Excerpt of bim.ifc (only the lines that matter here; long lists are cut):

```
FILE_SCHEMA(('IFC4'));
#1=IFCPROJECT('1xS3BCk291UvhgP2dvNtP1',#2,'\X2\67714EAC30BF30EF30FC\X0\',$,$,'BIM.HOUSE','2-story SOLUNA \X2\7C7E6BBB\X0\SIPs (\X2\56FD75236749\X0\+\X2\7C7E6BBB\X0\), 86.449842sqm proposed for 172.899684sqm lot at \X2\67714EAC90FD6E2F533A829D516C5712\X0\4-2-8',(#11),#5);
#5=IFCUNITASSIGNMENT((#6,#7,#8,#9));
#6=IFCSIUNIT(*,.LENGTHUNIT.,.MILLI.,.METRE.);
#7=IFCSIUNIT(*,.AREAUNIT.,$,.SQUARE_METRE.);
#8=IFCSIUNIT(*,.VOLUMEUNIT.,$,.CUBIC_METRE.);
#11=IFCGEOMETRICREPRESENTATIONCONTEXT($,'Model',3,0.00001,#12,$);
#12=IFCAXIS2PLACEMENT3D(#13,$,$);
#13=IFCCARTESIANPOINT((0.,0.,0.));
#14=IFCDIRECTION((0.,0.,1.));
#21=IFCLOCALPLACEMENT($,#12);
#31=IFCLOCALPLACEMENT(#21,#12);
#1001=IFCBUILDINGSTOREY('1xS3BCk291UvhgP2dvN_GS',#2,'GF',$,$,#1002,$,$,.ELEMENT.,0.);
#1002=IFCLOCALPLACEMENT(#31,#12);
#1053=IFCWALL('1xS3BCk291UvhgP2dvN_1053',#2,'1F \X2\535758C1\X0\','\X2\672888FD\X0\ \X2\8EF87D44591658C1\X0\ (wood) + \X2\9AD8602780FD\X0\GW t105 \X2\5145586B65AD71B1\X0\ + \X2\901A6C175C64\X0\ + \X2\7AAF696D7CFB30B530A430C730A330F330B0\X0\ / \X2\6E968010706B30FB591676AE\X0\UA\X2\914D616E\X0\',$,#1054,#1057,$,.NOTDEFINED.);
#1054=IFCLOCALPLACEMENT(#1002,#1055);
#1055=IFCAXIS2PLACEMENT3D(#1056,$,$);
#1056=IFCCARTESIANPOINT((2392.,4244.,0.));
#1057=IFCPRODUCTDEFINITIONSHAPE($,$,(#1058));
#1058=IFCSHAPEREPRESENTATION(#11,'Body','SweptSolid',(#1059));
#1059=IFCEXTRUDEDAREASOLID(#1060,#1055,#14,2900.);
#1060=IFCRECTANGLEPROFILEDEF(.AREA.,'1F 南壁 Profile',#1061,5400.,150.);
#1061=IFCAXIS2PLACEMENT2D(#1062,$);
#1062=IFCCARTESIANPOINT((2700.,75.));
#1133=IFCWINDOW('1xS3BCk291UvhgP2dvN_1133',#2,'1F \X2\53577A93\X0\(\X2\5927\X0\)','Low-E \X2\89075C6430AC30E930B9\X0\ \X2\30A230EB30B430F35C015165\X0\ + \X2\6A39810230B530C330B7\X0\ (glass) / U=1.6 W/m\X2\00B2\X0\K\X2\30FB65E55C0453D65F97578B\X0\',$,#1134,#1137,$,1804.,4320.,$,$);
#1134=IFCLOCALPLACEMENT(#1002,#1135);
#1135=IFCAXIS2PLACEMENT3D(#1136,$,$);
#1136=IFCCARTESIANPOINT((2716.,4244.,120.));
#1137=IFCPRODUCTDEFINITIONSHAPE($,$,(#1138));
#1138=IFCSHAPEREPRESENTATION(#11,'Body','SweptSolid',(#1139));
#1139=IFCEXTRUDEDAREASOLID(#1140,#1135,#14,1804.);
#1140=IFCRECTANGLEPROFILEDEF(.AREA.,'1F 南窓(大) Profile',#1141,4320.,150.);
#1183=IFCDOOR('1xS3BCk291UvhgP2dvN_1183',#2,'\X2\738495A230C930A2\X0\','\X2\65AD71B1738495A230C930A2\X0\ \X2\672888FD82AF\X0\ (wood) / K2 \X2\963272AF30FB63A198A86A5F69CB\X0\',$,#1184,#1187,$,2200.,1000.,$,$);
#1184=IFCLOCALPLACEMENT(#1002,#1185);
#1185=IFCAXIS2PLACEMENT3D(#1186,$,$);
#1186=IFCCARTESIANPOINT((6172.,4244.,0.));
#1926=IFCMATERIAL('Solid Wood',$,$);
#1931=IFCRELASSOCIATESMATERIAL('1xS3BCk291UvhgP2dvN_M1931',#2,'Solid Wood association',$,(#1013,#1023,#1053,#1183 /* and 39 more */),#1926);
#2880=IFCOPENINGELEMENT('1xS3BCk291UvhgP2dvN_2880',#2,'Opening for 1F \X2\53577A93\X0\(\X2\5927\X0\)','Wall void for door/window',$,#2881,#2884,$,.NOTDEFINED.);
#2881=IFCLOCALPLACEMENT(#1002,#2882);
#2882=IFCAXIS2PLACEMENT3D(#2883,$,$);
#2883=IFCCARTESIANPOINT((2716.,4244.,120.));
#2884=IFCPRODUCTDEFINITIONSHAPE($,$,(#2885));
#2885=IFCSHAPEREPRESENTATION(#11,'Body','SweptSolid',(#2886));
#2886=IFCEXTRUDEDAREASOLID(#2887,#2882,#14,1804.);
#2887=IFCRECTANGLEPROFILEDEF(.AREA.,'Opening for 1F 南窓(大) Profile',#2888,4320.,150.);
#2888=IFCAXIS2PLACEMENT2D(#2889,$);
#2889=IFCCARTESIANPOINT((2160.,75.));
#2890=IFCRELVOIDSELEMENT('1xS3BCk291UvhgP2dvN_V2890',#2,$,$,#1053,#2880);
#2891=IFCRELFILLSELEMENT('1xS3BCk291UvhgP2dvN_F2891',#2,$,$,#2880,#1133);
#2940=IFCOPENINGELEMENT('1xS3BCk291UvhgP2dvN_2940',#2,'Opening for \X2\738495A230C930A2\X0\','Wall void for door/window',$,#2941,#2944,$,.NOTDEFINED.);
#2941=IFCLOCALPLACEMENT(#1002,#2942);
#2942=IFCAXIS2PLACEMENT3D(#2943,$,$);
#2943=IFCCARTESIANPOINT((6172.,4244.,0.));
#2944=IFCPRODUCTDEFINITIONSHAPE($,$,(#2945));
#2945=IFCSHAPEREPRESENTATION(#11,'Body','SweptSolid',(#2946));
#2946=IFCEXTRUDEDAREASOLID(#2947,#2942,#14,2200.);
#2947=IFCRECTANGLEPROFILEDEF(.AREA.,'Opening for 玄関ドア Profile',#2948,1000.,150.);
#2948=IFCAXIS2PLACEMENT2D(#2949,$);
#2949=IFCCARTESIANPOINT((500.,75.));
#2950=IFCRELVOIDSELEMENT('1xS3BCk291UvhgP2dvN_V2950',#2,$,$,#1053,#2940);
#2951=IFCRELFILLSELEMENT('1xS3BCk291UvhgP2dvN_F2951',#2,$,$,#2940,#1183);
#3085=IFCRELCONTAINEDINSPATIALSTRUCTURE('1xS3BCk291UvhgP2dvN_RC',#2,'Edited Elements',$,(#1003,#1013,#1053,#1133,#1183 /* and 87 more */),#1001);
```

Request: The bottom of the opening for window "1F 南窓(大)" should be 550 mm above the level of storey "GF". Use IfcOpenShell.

```python
import numpy as np
import ifcopenshell
import ifcopenshell.api.geometry
import ifcopenshell.geom
import ifcopenshell.util.element
import ifcopenshell.util.placement
import ifcopenshell.util.shape
import ifcopenshell.util.unit

model = ifcopenshell.open("bim.ifc")
unit_scale = ifcopenshell.util.unit.calculate_unit_scale(model)

window = model.by_guid("1xS3BCk291UvhgP2dvN_1133")
opening = window.FillsVoids[0].RelatingOpeningElement
storey = ifcopenshell.util.element.get_container(window, ifc_class="IfcBuildingStorey")
level = ifcopenshell.util.placement.get_local_placement(storey.ObjectPlacement)[2, 3]

# The opening's origin need not be at the sill, so measure its lowest point.
shape = ifcopenshell.geom.create_shape(ifcopenshell.geom.settings(), opening)
bottom = ifcopenshell.util.shape.get_shape_bottom_elevation(shape, shape.geometry) / unit_scale
dz = level + 0.55 / unit_scale - bottom

shift = np.array([0.0, 0.0, dz])
# The window is not placed relative to its opening, so move both.
for product in (opening, window):
    matrix = ifcopenshell.util.placement.get_local_placement(product.ObjectPlacement)
    matrix[:3, 3] += shift
    ifcopenshell.api.geometry.edit_object_placement(model, product=product, matrix=matrix, is_si=False)

print(f"moved by {dz * unit_scale:+.3f} m")

model.write("bim-out.ifc")
```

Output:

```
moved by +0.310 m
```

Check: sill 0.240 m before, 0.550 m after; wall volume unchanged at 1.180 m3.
